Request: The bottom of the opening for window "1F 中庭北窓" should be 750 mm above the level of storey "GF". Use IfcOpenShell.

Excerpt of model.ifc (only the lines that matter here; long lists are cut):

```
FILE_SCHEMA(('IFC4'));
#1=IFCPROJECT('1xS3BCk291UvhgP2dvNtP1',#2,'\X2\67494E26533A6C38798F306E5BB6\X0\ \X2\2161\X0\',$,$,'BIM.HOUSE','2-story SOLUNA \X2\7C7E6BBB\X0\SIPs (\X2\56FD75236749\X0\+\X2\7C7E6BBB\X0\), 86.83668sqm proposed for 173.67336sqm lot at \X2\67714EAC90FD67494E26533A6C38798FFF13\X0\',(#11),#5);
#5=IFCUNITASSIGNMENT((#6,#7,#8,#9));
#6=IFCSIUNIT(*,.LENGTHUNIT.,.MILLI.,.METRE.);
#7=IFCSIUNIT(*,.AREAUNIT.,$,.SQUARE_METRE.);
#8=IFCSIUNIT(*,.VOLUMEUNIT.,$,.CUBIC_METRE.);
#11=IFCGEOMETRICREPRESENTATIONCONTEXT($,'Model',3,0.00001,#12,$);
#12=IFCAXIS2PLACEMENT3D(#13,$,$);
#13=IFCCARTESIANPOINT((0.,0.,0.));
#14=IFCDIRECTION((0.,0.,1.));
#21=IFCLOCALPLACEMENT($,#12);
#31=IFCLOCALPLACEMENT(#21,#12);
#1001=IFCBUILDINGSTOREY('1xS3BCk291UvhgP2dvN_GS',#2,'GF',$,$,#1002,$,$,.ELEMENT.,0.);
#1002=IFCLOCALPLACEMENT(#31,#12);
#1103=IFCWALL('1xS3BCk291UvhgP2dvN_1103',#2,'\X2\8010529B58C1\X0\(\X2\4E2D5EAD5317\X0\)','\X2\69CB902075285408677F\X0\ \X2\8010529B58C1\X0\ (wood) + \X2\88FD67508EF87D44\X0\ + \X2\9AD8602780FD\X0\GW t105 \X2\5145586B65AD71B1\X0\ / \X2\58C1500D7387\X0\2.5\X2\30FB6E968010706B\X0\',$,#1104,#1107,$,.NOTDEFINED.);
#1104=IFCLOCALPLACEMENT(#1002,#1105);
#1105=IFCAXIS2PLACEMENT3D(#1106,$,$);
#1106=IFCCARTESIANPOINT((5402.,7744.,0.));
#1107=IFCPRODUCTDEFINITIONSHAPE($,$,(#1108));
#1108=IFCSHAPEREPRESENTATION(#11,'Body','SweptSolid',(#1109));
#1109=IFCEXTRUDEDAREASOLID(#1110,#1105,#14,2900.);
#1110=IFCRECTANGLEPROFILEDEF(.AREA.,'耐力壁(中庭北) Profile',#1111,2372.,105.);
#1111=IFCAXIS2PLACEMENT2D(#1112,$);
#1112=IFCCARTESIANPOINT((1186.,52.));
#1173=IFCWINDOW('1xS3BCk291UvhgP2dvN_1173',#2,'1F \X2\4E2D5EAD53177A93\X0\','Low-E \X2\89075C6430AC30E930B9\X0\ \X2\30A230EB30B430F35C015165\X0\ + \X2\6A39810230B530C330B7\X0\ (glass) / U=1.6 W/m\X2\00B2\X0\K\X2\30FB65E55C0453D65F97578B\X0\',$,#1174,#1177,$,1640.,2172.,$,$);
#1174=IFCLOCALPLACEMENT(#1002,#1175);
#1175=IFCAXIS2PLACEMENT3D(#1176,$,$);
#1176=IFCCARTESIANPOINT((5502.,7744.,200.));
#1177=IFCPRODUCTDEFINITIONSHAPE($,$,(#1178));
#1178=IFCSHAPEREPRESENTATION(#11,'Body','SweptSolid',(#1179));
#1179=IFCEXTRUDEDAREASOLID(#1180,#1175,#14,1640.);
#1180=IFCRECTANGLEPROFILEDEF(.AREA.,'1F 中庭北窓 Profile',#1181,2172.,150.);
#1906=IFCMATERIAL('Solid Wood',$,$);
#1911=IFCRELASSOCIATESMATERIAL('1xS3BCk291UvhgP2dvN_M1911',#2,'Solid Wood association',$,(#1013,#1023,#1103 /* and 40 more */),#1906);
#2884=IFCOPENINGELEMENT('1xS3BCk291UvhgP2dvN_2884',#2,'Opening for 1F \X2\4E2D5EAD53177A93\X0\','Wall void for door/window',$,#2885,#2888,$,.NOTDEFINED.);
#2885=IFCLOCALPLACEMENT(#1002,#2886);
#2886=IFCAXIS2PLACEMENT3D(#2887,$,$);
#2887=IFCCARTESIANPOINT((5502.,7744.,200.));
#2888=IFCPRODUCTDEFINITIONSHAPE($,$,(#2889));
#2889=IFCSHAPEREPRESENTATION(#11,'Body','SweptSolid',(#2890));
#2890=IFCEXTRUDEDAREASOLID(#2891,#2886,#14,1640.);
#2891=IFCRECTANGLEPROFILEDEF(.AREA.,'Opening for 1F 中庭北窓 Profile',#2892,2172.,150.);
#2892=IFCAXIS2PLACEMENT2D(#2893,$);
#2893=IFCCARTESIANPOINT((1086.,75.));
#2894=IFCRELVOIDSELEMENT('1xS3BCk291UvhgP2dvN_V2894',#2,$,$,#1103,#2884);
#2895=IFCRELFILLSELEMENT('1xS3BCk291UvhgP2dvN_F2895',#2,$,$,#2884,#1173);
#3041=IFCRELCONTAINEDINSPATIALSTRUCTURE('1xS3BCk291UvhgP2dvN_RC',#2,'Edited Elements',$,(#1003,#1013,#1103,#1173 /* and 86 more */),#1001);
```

```python
import numpy as np
import ifcopenshell
import ifcopenshell.api.geometry
import ifcopenshell.geom
import ifcopenshell.util.element
import ifcopenshell.util.placement
import ifcopenshell.util.shape
import ifcopenshell.util.unit

model = ifcopenshell.open("model.ifc")
unit_scale = ifcopenshell.util.unit.calculate_unit_scale(model)

window = model.by_guid("1xS3BCk291UvhgP2dvN_1173")
opening = window.FillsVoids[0].RelatingOpeningElement
storey = ifcopenshell.util.element.get_container(window, ifc_class="IfcBuildingStorey")
level = ifcopenshell.util.placement.get_local_placement(storey.ObjectPlacement)[2, 3]

# The opening's origin need not be at the sill, so measure its lowest point.
shape = ifcopenshell.geom.create_shape(ifcopenshell.geom.settings(), opening)
bottom = ifcopenshell.util.shape.get_shape_bottom_elevation(shape, shape.geometry) / unit_scale
dz = level + 0.75 / unit_scale - bottom

shift = np.array([0.0, 0.0, dz])
# The window is not placed relative to its opening, so move both.
for product in (opening, window):
    matrix = ifcopenshell.util.placement.get_local_placement(product.ObjectPlacement)
    matrix[:3, 3] += shift
    ifcopenshell.api.geometry.edit_object_placement(model, product=product, matrix=matrix, is_si=False)

print(f"moved by {dz * unit_scale:+.3f} m")

model.write("model_updated.ifc")
```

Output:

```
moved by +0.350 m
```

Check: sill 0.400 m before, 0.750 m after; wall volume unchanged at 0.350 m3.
